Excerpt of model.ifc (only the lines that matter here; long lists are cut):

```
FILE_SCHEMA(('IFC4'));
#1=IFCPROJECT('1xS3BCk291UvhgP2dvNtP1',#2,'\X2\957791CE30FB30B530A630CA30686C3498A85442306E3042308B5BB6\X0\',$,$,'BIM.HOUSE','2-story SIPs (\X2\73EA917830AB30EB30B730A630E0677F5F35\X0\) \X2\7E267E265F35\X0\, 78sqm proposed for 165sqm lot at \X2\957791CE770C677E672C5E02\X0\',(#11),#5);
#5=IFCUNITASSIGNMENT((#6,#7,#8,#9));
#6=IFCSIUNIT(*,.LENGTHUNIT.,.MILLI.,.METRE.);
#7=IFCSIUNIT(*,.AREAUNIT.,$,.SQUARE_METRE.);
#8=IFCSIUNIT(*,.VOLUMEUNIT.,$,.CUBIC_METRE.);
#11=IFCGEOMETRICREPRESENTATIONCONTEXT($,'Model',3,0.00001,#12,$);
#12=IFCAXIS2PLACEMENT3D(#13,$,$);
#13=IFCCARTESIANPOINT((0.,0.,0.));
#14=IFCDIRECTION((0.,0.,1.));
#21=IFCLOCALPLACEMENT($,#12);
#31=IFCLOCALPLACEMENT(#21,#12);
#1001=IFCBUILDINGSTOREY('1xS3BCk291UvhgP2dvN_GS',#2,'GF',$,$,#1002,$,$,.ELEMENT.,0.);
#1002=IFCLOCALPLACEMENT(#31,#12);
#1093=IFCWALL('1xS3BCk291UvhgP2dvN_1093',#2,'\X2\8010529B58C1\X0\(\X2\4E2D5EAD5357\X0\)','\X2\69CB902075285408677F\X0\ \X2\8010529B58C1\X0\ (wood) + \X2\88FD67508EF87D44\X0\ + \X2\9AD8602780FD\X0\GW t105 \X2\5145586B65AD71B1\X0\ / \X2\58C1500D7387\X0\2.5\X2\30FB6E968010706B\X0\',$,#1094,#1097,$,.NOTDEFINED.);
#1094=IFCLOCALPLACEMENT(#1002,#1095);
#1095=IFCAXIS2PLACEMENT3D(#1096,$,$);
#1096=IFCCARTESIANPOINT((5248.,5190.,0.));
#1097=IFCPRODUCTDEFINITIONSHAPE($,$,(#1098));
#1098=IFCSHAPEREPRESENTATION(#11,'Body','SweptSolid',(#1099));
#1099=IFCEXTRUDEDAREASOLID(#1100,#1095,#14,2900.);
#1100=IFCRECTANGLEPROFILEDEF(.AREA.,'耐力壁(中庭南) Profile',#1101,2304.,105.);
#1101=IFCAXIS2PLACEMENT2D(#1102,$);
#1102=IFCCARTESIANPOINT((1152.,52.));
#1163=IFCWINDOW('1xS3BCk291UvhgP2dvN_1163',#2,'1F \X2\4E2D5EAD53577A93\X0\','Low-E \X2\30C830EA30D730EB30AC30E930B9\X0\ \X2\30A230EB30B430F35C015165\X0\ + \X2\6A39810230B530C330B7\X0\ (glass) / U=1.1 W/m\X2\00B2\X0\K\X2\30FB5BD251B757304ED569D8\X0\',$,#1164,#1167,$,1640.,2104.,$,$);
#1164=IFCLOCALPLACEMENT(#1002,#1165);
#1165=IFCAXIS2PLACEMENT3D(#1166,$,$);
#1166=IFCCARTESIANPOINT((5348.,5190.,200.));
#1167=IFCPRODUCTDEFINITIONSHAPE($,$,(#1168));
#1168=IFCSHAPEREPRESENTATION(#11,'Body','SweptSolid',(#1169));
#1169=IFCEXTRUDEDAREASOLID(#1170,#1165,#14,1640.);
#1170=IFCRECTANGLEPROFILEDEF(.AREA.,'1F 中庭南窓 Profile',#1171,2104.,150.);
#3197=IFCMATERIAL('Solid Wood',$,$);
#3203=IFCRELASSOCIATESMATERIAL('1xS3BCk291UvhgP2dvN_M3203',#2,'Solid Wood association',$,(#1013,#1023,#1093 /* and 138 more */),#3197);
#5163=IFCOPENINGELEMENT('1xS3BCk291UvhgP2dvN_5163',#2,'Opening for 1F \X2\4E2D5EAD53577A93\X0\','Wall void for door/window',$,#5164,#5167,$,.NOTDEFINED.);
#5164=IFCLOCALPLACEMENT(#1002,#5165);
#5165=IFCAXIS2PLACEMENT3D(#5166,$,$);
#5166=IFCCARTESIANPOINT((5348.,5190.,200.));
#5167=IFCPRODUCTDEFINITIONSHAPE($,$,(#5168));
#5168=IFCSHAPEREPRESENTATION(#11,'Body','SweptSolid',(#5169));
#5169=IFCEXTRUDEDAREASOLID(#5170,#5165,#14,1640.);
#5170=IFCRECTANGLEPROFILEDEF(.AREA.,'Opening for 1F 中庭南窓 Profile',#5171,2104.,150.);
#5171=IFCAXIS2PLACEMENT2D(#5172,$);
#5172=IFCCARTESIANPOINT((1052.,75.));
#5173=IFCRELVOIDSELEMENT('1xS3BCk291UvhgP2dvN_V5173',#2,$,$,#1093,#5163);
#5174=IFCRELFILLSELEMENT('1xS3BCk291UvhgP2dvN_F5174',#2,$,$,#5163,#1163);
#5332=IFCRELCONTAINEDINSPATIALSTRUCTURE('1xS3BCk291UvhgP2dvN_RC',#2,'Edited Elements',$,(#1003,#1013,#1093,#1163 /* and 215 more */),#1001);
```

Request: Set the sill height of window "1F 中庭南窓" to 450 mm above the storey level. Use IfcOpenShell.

```python
import numpy as np
import ifcopenshell
import ifcopenshell.api.geometry
import ifcopenshell.geom
import ifcopenshell.util.element
import ifcopenshell.util.placement
import ifcopenshell.util.shape
import ifcopenshell.util.unit

model = ifcopenshell.open("model.ifc")
unit_scale = ifcopenshell.util.unit.calculate_unit_scale(model)

window = model.by_guid("1xS3BCk291UvhgP2dvN_1163")
opening = window.FillsVoids[0].RelatingOpeningElement
storey = ifcopenshell.util.element.get_container(window, ifc_class="IfcBuildingStorey")
level = ifcopenshell.util.placement.get_local_placement(storey.ObjectPlacement)[2, 3]

# The opening's origin need not be at the sill, so measure its lowest point.
shape = ifcopenshell.geom.create_shape(ifcopenshell.geom.settings(), opening)
bottom = ifcopenshell.util.shape.get_shape_bottom_elevation(shape, shape.geometry) / unit_scale
dz = level + 450.0 - bottom

shift = np.array([0.0, 0.0, dz])
# The window is not placed relative to its opening, so move both.
for product in (opening, window):
    matrix = ifcopenshell.util.placement.get_local_placement(product.ObjectPlacement)
    matrix[:3, 3] += shift
    ifcopenshell.api.geometry.edit_object_placement(model, product=product, matrix=matrix, is_si=False)

print(f"moved by {dz * unit_scale:+.3f} m")

model.write("model_rev.ifc")
```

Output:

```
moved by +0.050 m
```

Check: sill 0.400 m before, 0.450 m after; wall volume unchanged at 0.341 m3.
